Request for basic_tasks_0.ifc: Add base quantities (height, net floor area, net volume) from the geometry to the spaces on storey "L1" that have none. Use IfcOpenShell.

First a look at what the model holds.

```python
import ifcopenshell
import ifcopenshell.util.element
import ifcopenshell.util.unit

model = ifcopenshell.open("basic_tasks_0.ifc")
print(model.schema)
for unit_type in ("LENGTHUNIT", "AREAUNIT", "VOLUMEUNIT"):
    print(unit_type, ifcopenshell.util.unit.calculate_unit_scale(model, unit_type))
storey = next(s for s in model.by_type("IfcBuildingStorey") if s.Name == "L1")
spaces = [e for e in ifcopenshell.util.element.get_decomposition(storey) if e.is_a("IfcSpace")]
for e in sorted(spaces, key=lambda e: e.id()):
    print(e.id(), e.is_a(), e.Name, list(ifcopenshell.util.element.get_psets(e, qtos_only=True)), sep=" | ")
```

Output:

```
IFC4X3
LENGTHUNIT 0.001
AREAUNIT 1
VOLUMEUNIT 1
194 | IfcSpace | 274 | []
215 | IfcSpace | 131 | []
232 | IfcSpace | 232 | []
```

```python
import ifcopenshell
import ifcopenshell.api.pset
import ifcopenshell.geom
import ifcopenshell.util.element
import ifcopenshell.util.shape
import ifcopenshell.util.unit

model = ifcopenshell.open("basic_tasks_0.ifc")
unit_scale = ifcopenshell.util.unit.calculate_unit_scale(model)
area_scale = ifcopenshell.util.unit.calculate_unit_scale(model, "AREAUNIT")
volume_scale = ifcopenshell.util.unit.calculate_unit_scale(model, "VOLUMEUNIT")
settings = ifcopenshell.geom.settings()

storey = next(s for s in model.by_type("IfcBuildingStorey") if s.Name == "L1")
spaces = [e for e in ifcopenshell.util.element.get_decomposition(storey) if e.is_a("IfcSpace")]

for e in sorted(spaces, key=lambda e: e.id()):
    if ifcopenshell.util.element.get_psets(e, qtos_only=True, should_inherit=False):
        continue
    # Geometry comes back in metres, in the element's own axes.
    shape = ifcopenshell.geom.create_shape(settings, e)
    values = {
        "Height": ifcopenshell.util.shape.get_z(shape.geometry) / unit_scale,
        "NetFloorArea": ifcopenshell.util.shape.get_footprint_area(shape.geometry) / area_scale,
        "NetVolume": ifcopenshell.util.shape.get_volume(shape.geometry) / volume_scale,
    }
    qto = ifcopenshell.api.pset.add_qto(model, product=e, name="Qto_SpaceBaseQuantities")
    ifcopenshell.api.pset.edit_qto(model, qto=qto, properties=values)
    print(e.id(), {k: round(v, 3) for k, v in values.items()})

model.write("basic_tasks_0_v2.ifc")
```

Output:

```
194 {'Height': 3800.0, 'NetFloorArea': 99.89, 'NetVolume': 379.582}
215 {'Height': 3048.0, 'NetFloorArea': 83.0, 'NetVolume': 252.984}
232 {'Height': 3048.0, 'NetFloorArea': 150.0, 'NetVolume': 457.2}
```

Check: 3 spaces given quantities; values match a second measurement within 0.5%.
